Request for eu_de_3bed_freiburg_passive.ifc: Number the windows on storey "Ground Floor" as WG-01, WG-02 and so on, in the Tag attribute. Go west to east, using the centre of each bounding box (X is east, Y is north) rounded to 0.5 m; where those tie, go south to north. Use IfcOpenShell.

First a look at what the model holds.

```python
import ifcopenshell
import ifcopenshell.util.element
import ifcopenshell.util.placement

model = ifcopenshell.open("eu_de_3bed_freiburg_passive.ifc")
print(model.schema)
storey = next(s for s in model.by_type("IfcBuildingStorey") if s.Name == "Ground Floor")
windows = [e for e in ifcopenshell.util.element.get_decomposition(storey) if e.is_a("IfcWindow")]
for e in sorted(windows, key=lambda e: e.id()):
    origin = ifcopenshell.util.placement.get_local_placement(e.ObjectPlacement)[:3, 3]
    print(e.id(), e.Tag, e.Name, origin.round(2) + 0.0, sep=" | ")
```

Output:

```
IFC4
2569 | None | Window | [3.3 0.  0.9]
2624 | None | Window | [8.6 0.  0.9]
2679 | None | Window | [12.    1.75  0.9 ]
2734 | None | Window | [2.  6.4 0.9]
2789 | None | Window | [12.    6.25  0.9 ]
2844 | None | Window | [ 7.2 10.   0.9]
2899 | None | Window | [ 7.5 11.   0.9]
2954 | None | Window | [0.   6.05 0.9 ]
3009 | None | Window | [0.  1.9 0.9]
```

```python
import ifcopenshell
import ifcopenshell.geom
import ifcopenshell.util.element
import ifcopenshell.util.shape

model = ifcopenshell.open("eu_de_3bed_freiburg_passive.ifc")
settings = ifcopenshell.geom.settings()
settings.set("use-world-coords", True)


def centre(element):
    shape = ifcopenshell.geom.create_shape(settings, element)
    return ifcopenshell.util.shape.get_bbox_centroid(shape.geometry)


storey = next(s for s in model.by_type("IfcBuildingStorey") if s.Name == "Ground Floor")
windows = [e for e in ifcopenshell.util.element.get_decomposition(storey) if e.is_a("IfcWindow")]

# Insertion points can sit at a corner or the storey origin, so sort by the geometry (in metres).
centres = {e: centre(e) for e in windows}
windows.sort(key=lambda e: (round(centres[e][0] / 0.5), centres[e][1]))

for i, e in enumerate(windows, start=1):
    number = f"WG-{i:02d}"
    e.Tag = number
    print(e.id(), number)

model.write("eu_de_3bed_freiburg_passive_v2.ifc")
```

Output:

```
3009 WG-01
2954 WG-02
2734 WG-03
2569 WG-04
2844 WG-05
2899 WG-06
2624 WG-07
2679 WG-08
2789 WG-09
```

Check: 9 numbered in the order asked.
